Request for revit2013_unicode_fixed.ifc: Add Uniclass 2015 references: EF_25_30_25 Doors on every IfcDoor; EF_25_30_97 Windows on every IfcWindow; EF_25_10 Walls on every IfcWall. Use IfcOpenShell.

First a look at what the model holds.

```python
import ifcopenshell

model = ifcopenshell.open("revit2013_unicode_fixed.ifc")
print(model.schema)
print("classifications:", [c.Name for c in model.by_type("IfcClassification")])
for ifc_class in ("IfcDoor", "IfcRoof", "IfcStair", "IfcWall", "IfcWindow"):
    print(ifc_class, len(model.by_type(ifc_class)))
```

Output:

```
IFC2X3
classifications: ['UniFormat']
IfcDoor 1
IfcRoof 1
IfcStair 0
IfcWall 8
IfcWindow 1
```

```python
import ifcopenshell
import ifcopenshell.api.classification

model = ifcopenshell.open("revit2013_unicode_fixed.ifc")

# IFC2X3 requires Source and Edition and has no link from the project to the system.
system = model.create_entity("IfcClassification", Source="NBS", Edition="2015", Name="Uniclass 2015")

codes = {
    "IfcDoor": ("EF_25_30_25", "Doors"),
    "IfcWindow": ("EF_25_30_97", "Windows"),
    "IfcWall": ("EF_25_10", "Walls"),
}
for ifc_class, (code, name) in codes.items():
    products = model.by_type(ifc_class)
    ifcopenshell.api.classification.add_reference(
        model, products=products, classification=system, identification=code, name=name
    )
    print(code, len(products))

model.write("revit2013_unicode_fixed_rev.ifc")
```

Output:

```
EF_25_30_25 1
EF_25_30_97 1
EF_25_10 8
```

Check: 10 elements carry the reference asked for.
